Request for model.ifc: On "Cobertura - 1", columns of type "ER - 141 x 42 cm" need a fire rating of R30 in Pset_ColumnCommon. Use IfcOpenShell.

First a look at what the model holds.

```python
import ifcopenshell
import ifcopenshell.util.element

model = ifcopenshell.open("model.ifc")
print(model.schema)
storey = next(s for s in model.by_type("IfcBuildingStorey") if s.Name == "Cobertura - 1")
columns = [e for e in ifcopenshell.util.element.get_decomposition(storey) if e.is_a("IfcColumn")]
seen = {}
for e in columns:
    element_type = ifcopenshell.util.element.get_type(e)
    key = (element_type.Name if element_type != e and element_type else None, ifcopenshell.util.element.get_pset(e, "Pset_ColumnCommon", "FireRating"))
    seen[key] = seen.get(key, 0) + 1
for (name, value), count in sorted(seen.items(), key=str):
    print(count, "x", name, "|", value)
```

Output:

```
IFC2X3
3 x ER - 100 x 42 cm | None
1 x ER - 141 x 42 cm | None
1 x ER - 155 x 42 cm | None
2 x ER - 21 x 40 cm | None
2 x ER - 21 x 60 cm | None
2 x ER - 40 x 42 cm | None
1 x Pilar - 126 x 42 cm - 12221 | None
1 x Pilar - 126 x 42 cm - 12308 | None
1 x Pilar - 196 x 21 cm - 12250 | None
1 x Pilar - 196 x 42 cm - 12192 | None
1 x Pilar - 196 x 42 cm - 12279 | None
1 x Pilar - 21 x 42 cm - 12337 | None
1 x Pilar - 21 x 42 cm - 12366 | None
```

```python
import ifcopenshell
import ifcopenshell.api.pset
import ifcopenshell.util.element

model = ifcopenshell.open("model.ifc")

storey = next(s for s in model.by_type("IfcBuildingStorey") if s.Name == "Cobertura - 1")
columns = [e for e in ifcopenshell.util.element.get_decomposition(storey) if e.is_a("IfcColumn")]

count = 0
for e in columns:
    element_type = ifcopenshell.util.element.get_type(e)
    if element_type in (None, e) or element_type.Name != "ER - 141 x 42 cm":
        continue
    # add_pset returns the element's existing set when there is one.
    pset = ifcopenshell.api.pset.add_pset(model, product=e, name="Pset_ColumnCommon")
    ifcopenshell.api.pset.edit_pset(model, pset=pset, properties={"FireRating": "R30"})
    count += 1

print(count, "columns updated")

model.write("model_edited.ifc")
```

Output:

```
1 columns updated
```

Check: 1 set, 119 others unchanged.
